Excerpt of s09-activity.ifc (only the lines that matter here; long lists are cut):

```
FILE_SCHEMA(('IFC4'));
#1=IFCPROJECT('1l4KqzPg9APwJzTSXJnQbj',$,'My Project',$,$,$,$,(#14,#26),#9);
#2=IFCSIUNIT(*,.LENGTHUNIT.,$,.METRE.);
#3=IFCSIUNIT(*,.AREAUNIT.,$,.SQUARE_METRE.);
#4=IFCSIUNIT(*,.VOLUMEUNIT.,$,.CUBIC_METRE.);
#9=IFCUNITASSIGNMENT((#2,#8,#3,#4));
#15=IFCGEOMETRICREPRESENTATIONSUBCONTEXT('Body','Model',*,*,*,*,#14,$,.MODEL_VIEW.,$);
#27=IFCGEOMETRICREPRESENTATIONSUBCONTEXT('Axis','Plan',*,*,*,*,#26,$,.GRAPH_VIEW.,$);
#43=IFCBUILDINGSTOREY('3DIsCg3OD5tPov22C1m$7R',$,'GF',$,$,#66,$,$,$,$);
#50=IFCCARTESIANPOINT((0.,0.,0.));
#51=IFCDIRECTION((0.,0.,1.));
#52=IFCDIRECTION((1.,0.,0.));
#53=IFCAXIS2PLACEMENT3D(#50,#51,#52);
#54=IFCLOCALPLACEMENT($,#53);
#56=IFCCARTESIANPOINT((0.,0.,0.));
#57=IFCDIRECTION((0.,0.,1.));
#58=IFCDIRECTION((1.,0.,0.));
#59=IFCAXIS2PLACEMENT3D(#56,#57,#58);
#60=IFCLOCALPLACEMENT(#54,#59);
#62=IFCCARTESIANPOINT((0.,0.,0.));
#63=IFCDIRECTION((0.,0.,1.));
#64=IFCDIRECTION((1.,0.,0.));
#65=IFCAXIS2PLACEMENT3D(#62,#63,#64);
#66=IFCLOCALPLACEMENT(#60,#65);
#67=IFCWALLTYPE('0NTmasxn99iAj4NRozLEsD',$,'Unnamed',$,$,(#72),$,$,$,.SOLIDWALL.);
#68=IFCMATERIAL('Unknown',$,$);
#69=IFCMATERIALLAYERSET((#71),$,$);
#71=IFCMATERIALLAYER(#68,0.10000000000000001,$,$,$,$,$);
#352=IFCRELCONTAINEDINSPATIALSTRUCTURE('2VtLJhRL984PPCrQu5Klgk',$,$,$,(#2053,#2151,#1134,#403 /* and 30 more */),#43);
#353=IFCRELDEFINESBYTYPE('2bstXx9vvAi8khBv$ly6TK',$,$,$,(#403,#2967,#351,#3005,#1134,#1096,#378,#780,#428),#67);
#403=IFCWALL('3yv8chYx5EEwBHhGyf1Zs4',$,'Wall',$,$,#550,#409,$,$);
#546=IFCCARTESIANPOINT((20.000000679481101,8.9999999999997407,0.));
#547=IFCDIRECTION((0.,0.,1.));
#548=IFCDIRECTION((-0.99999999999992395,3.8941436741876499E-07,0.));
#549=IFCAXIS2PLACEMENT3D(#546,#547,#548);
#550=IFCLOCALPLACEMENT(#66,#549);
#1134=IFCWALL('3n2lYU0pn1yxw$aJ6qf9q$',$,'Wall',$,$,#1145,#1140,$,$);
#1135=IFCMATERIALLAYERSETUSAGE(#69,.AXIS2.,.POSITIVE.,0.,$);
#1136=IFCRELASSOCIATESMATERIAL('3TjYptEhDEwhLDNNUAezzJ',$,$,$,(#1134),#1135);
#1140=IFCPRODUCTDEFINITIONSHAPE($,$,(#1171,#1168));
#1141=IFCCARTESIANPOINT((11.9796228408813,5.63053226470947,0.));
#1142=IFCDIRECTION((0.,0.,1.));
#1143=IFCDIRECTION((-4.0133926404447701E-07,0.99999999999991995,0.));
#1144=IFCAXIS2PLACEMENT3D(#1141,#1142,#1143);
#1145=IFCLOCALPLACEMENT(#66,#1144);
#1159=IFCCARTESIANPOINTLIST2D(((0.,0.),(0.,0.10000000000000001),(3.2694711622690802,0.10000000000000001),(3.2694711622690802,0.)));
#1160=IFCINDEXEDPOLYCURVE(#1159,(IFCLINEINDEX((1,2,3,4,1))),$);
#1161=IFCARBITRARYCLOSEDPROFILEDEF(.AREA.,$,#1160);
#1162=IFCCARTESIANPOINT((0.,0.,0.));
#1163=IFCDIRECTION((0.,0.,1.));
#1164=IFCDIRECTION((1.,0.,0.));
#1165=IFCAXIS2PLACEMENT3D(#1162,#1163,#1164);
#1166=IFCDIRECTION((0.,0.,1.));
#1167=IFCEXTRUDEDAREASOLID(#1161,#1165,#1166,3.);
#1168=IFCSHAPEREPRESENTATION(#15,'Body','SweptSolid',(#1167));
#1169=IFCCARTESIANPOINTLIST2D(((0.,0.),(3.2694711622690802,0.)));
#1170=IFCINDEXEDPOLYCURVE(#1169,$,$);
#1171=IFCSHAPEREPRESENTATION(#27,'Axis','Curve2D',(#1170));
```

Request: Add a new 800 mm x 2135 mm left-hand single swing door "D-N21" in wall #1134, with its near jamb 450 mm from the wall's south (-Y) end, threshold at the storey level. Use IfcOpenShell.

```python
import numpy as np
import ifcopenshell
import ifcopenshell.api.feature
import ifcopenshell.api.geometry
import ifcopenshell.api.root
import ifcopenshell.api.spatial
import ifcopenshell.geom
import ifcopenshell.util.element
import ifcopenshell.util.placement
import ifcopenshell.util.representation
import ifcopenshell.util.shape
import ifcopenshell.util.unit

model = ifcopenshell.open("s09-activity.ifc")
unit_scale = ifcopenshell.util.unit.calculate_unit_scale(model)
settings = ifcopenshell.geom.settings()


def volume(element):
    """Net volume in cubic metres, openings subtracted."""
    shape = ifcopenshell.geom.create_shape(settings, element)
    return ifcopenshell.util.shape.get_volume(shape.geometry)


wall = model.by_guid("3n2lYU0pn1yxw$aJ6qf9q$")
storey = ifcopenshell.util.element.get_container(wall, ifc_class="IfcBuildingStorey")
context = ifcopenshell.util.representation.get_context(model, "Model", "Body", "MODEL_VIEW")
before = volume(wall)

width, height, from_end, sill = 0.8, 2.135, 0.45, 0.0  # metres

# The wall runs along its own X axis, and the end named is its -X end.
wall_shape = ifcopenshell.geom.create_shape(settings, wall)
x, y, z = ifcopenshell.util.shape.get_vertices(wall_shape.geometry).T
start = x.min() + from_end
face, thickness = float(y.min()), float(y.max() - y.min())
wall_matrix = ifcopenshell.util.placement.get_local_placement(wall.ObjectPlacement)
level = ifcopenshell.util.placement.get_local_placement(storey.ObjectPlacement)[2, 3]


def in_wall(x, y):
    """Placement at x, y metres in the wall's axes, at sill height."""
    matrix = wall_matrix.copy()
    matrix[:, 3] = wall_matrix @ np.array([x / unit_scale, y / unit_scale, 0.0, 1.0])
    matrix[2, 3] = level + sill / unit_scale
    return matrix


# Opening: a box that overshoots both wall faces by 50 mm.
opening = ifcopenshell.api.root.create_entity(model, ifc_class="IfcOpeningElement", predefined_type="OPENING")
box = ifcopenshell.api.geometry.add_wall_representation(
    model, context=context, length=width, height=height, thickness=thickness + 0.1
)
ifcopenshell.api.geometry.assign_representation(model, product=opening, representation=box)
ifcopenshell.api.geometry.edit_object_placement(model, product=opening, matrix=in_wall(start, face - 0.05), is_si=False)
ifcopenshell.api.feature.add_feature(model, feature=opening, element=wall)

door = ifcopenshell.api.root.create_entity(model, ifc_class="IfcDoor", name="D-N21", predefined_type="DOOR")
door.OverallWidth, door.OverallHeight = width / unit_scale, height / unit_scale
door.OperationType = "SINGLE_SWING_LEFT"
body = ifcopenshell.api.geometry.add_door_representation(
    model,
    context=context,
    overall_width=door.OverallWidth,
    overall_height=door.OverallHeight,
    operation_type="SINGLE_SWING_LEFT",
    lining_properties={"LiningDepth": thickness / unit_scale, "ThresholdDepth": thickness / unit_scale},
)
ifcopenshell.api.geometry.assign_representation(model, product=door, representation=body)
ifcopenshell.api.spatial.assign_container(model, products=[door], relating_structure=storey)
ifcopenshell.api.feature.add_filling(model, opening=opening, element=door)

# The lining spans the wall, so the door starts at the wall face.
ifcopenshell.api.geometry.edit_object_placement(model, product=door, matrix=in_wall(start, face), is_si=False)

after = volume(wall)

print(f"wall volume {before:.3f} -> {after:.3f} m3")

model.write("s09-activity-out.ifc")
```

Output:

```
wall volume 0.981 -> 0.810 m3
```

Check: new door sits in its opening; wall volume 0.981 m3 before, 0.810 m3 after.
